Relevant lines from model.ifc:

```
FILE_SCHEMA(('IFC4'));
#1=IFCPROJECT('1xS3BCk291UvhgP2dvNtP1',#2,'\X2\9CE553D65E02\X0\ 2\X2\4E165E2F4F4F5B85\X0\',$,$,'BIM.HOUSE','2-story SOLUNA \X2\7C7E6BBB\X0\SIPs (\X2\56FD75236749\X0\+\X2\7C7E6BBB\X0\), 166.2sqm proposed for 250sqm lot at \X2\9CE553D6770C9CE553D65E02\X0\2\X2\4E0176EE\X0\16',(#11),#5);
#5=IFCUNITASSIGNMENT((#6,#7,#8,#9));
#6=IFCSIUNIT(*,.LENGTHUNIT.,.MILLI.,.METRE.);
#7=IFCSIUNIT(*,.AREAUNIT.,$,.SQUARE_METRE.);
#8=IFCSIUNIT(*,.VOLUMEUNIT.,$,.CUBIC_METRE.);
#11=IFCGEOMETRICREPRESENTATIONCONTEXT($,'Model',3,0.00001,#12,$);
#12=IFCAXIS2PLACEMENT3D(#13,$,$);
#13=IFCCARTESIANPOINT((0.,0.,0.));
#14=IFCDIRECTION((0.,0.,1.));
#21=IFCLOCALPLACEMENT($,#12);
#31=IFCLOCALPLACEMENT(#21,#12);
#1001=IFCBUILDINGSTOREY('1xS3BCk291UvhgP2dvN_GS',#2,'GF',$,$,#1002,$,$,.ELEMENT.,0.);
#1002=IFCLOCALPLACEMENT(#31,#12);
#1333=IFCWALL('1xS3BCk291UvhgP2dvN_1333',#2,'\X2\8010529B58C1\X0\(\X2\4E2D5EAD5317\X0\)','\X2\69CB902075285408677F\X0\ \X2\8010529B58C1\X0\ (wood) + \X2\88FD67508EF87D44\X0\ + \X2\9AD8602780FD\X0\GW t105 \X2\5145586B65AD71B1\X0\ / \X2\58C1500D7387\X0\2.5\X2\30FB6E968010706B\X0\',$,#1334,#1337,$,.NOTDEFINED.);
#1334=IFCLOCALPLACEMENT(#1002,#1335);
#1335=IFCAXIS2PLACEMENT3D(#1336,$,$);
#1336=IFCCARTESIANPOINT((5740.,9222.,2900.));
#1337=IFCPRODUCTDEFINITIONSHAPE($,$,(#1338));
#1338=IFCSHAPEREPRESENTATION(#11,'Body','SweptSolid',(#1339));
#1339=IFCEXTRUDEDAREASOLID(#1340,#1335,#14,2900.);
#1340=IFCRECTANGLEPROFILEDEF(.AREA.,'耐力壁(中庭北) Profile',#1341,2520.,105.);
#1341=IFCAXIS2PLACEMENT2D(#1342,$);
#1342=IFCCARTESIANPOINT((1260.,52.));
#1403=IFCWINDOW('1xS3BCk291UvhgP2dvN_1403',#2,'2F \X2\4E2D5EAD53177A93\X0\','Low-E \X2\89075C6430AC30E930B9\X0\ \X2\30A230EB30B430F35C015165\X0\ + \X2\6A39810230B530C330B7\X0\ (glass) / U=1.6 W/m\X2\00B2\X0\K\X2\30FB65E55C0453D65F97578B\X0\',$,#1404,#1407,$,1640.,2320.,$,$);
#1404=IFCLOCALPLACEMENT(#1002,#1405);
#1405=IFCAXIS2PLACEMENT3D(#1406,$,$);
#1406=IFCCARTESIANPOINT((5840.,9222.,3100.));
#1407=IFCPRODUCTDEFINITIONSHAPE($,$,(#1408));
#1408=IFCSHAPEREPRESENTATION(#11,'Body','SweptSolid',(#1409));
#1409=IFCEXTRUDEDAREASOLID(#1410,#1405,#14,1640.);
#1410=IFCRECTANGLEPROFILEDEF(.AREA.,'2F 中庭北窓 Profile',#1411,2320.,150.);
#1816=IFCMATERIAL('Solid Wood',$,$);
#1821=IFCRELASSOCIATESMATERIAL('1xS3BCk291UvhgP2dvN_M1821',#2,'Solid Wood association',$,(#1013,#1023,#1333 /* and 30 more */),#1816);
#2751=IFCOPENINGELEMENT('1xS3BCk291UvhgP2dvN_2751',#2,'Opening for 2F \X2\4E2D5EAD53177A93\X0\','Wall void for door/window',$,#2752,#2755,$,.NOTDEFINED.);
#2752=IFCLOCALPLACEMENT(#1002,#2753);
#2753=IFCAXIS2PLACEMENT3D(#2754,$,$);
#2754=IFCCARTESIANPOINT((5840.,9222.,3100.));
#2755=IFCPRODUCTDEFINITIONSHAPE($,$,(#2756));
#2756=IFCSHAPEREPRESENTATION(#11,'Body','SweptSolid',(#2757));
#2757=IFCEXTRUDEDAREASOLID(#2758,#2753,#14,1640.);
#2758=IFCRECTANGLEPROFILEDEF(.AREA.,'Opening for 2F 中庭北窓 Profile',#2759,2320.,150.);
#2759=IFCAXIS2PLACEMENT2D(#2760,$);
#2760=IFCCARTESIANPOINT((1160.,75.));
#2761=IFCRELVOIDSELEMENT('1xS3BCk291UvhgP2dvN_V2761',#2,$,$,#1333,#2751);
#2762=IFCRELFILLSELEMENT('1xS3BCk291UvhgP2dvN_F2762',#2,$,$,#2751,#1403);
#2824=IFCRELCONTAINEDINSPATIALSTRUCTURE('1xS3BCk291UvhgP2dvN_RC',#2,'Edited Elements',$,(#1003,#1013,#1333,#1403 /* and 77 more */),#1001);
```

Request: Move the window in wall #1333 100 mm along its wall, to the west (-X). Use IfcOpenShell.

```python
import ifcopenshell
import ifcopenshell.api.geometry
import ifcopenshell.util.placement
import ifcopenshell.util.unit

model = ifcopenshell.open("model.ifc")
unit_scale = ifcopenshell.util.unit.calculate_unit_scale(model)

window = model.by_guid("1xS3BCk291UvhgP2dvN_1403")
opening = window.FillsVoids[0].RelatingOpeningElement
wall = opening.VoidsElements[0].RelatingBuildingElement

wall_matrix = ifcopenshell.util.placement.get_local_placement(wall.ObjectPlacement)
shift = wall_matrix[:3, 0] * -0.1 / unit_scale
before = ifcopenshell.util.placement.get_local_placement(window.ObjectPlacement)[:3, 3].copy()

# The window is not placed relative to its opening, so move both.
for product in (opening, window):
    matrix = ifcopenshell.util.placement.get_local_placement(product.ObjectPlacement)
    matrix[:3, 3] += shift
    ifcopenshell.api.geometry.edit_object_placement(model, product=product, matrix=matrix, is_si=False)

after = ifcopenshell.util.placement.get_local_placement(window.ObjectPlacement)[:3, 3]
print("window moved by", (after - before).round(3) + 0.0)

model.write("model_rev.ifc")
```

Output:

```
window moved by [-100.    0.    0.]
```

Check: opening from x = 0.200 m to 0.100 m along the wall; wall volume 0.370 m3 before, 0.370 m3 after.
